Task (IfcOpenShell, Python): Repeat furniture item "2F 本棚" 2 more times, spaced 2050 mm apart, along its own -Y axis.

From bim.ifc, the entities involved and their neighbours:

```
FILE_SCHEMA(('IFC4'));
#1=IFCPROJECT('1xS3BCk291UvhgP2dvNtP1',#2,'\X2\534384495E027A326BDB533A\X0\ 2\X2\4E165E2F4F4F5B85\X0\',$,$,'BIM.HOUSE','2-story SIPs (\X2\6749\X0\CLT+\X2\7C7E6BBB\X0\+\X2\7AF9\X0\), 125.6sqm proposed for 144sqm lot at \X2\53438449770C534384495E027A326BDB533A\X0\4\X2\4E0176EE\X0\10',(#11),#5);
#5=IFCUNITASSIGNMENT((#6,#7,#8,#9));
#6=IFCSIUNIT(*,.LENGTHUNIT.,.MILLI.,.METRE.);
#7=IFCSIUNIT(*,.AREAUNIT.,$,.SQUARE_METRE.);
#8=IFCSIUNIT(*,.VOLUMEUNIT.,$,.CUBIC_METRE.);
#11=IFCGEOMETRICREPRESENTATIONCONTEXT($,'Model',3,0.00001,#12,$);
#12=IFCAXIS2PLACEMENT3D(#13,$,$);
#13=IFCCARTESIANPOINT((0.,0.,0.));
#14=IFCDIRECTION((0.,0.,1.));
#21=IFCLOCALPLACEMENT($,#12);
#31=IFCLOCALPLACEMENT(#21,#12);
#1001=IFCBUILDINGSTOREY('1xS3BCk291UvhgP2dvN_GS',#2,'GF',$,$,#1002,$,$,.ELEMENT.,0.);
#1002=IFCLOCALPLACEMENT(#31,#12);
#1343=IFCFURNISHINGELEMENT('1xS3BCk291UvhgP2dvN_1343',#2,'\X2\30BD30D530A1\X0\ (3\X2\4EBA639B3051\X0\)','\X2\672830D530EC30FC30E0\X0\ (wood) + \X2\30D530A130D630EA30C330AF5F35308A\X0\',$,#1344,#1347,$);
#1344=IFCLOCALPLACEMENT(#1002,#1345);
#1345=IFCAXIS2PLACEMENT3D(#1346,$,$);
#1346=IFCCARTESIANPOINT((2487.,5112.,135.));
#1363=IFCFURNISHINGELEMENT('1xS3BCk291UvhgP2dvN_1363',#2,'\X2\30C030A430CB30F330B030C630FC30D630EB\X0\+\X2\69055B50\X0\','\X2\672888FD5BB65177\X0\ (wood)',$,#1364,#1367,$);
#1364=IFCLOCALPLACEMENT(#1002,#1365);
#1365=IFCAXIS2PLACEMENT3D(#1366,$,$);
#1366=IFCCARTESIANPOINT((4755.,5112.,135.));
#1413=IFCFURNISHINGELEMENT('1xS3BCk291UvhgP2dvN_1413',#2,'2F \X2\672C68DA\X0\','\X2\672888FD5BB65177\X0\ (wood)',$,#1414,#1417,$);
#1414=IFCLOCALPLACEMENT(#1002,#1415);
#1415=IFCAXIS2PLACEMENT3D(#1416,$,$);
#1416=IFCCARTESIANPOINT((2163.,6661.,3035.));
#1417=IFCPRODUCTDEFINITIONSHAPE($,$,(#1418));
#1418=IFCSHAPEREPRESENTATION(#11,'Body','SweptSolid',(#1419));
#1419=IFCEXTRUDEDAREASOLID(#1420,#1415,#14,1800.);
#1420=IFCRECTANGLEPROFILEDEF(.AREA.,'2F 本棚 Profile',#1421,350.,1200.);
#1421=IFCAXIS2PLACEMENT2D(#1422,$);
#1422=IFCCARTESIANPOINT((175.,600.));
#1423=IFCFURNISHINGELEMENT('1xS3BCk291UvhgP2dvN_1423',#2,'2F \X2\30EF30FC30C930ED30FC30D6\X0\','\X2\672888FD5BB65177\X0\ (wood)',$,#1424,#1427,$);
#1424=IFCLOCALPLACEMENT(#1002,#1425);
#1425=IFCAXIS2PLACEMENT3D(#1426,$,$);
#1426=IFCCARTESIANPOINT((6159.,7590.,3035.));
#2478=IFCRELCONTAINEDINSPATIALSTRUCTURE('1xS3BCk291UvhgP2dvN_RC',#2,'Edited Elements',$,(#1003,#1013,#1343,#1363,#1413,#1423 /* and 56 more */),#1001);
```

```python
import ifcopenshell
import ifcopenshell.api.geometry
import ifcopenshell.api.root
import ifcopenshell.util.element
import ifcopenshell.util.placement
import ifcopenshell.util.unit

model = ifcopenshell.open("bim.ifc")
unit_scale = ifcopenshell.util.unit.calculate_unit_scale(model)


def reuse_history(source, copy):
    """copy_class also copies each property set's owner history, people and application; keep the originals."""
    for rel in copy.IsDefinedBy:
        if rel.is_a("IfcRelDefinesByProperties") and (history := rel.RelatingPropertyDefinition.OwnerHistory):
            rel.RelatingPropertyDefinition.OwnerHistory = source.OwnerHistory
            ifcopenshell.util.element.remove_deep2(model, history)


source = model.by_id(1413)
base = ifcopenshell.util.placement.get_local_placement(source.ObjectPlacement)
step = -base[:3, 1] * 2.05 / unit_scale

for i in range(1, 3):
    copy = ifcopenshell.api.root.copy_class(model, product=source)
    copy.Representation = ifcopenshell.util.element.copy_deep(
        model, source.Representation, exclude=["IfcGeometricRepresentationContext", "IfcRepresentationMap"]
    )
    reuse_history(source, copy)
    matrix = base.copy()
    matrix[:3, 3] += i * step
    print("added at", matrix[:3, 3].round(3) + 0.0)
    ifcopenshell.api.geometry.edit_object_placement(model, product=copy, matrix=matrix, is_si=False)

model.write("bim_rev.ifc")
```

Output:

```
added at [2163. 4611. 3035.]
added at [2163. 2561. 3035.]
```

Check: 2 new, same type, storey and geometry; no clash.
